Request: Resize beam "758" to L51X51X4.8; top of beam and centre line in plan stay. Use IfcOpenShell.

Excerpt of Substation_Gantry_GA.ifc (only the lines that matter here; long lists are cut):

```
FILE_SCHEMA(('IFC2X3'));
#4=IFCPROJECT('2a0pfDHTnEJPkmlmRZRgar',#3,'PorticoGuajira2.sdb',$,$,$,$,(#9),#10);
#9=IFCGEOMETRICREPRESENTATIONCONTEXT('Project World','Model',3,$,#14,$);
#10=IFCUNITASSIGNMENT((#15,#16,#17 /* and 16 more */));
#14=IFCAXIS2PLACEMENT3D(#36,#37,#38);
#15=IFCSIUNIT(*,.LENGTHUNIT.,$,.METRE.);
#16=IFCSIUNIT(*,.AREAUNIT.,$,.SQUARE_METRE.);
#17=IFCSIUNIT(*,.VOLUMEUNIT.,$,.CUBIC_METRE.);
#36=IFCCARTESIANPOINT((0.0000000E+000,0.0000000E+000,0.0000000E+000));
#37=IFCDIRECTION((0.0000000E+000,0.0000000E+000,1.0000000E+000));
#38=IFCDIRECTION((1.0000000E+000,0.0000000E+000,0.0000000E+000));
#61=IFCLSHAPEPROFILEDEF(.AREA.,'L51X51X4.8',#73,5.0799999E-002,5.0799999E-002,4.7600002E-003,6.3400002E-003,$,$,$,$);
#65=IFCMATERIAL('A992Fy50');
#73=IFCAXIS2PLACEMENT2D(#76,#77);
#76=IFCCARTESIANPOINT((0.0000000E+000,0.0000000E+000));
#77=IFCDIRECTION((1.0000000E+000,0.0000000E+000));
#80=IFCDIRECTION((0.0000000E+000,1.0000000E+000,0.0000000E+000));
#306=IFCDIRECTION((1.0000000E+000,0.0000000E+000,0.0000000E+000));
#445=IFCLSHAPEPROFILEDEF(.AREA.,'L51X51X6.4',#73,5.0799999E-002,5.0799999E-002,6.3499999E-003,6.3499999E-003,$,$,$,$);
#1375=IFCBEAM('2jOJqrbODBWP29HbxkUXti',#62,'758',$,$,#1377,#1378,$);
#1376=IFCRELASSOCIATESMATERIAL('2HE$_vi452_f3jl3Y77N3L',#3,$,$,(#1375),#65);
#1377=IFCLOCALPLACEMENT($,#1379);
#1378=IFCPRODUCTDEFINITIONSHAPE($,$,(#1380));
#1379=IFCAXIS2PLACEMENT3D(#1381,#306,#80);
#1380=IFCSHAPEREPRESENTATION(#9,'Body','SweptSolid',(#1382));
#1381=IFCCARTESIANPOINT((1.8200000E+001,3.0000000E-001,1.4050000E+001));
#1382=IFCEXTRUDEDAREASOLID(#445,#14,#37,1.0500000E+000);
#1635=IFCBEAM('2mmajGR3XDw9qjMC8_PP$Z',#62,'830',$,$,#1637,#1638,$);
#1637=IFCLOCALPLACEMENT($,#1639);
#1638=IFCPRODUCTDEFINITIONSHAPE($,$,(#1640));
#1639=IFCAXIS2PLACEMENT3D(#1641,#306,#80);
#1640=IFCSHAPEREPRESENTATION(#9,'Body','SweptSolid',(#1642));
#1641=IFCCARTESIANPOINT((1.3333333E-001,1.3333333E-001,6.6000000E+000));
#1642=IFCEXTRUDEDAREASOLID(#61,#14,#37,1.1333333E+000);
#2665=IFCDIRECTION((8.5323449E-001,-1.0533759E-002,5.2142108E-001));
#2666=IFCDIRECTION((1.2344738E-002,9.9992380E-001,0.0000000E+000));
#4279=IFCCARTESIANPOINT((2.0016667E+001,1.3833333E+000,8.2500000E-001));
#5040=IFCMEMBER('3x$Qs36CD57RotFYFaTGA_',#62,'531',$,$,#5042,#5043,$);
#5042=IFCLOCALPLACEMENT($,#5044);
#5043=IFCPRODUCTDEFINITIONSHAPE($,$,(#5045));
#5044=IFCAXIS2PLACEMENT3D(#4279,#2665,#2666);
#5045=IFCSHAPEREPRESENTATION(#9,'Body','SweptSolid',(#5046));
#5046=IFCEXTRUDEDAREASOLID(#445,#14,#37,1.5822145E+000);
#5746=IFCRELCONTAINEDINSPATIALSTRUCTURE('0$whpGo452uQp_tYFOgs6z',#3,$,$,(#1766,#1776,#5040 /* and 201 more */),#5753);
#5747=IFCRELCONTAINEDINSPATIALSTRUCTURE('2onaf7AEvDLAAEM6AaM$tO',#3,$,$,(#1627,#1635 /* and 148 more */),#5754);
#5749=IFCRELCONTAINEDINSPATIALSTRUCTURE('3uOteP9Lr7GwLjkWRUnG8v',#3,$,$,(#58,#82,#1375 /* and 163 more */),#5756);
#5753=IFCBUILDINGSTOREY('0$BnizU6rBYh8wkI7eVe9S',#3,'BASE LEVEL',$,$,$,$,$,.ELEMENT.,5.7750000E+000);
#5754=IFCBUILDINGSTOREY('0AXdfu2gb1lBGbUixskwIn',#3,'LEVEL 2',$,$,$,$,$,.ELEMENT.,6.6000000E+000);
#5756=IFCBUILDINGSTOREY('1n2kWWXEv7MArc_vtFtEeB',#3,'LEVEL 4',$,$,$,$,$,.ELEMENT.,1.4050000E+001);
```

```python
import ifcopenshell
import ifcopenshell.util.element

model = ifcopenshell.open("Substation_Gantry_GA.ifc")

member = model.by_id(1375)
source = next(p for p in model.by_type("IfcLShapeProfileDef") if p.ProfileName == "L51X51X4.8")

body = next(r for r in member.Representation.Representations if r.RepresentationIdentifier == "Body")
solid = body.Items[0]
old_profile = solid.SweptArea

# Copy the section's sizes but keep this member's own profile position.
profile = ifcopenshell.util.element.copy(model, source)
# Profiles are centred, so shift by half the change in depth to hold the top.
shift = (old_profile.Depth - profile.Depth) / 2
x, y = old_profile.Position.Location.Coordinates
up = (0.0, 1.0)  # upwards, in the solid's own plane
location = model.createIfcCartesianPoint((x + up[0] * shift, y + up[1] * shift))
profile.Position = model.createIfcAxis2Placement2D(location, old_profile.Position.RefDirection)
solid.SweptArea = profile
if not model.get_total_inverses(old_profile):
    ifcopenshell.util.element.remove_deep2(model, old_profile)

print(solid.SweptArea)

model.write("Substation_Gantry_GA-out.ifc")
```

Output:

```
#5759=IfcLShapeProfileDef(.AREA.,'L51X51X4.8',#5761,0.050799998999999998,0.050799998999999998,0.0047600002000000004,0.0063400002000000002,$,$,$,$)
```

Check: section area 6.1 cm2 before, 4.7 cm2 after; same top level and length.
